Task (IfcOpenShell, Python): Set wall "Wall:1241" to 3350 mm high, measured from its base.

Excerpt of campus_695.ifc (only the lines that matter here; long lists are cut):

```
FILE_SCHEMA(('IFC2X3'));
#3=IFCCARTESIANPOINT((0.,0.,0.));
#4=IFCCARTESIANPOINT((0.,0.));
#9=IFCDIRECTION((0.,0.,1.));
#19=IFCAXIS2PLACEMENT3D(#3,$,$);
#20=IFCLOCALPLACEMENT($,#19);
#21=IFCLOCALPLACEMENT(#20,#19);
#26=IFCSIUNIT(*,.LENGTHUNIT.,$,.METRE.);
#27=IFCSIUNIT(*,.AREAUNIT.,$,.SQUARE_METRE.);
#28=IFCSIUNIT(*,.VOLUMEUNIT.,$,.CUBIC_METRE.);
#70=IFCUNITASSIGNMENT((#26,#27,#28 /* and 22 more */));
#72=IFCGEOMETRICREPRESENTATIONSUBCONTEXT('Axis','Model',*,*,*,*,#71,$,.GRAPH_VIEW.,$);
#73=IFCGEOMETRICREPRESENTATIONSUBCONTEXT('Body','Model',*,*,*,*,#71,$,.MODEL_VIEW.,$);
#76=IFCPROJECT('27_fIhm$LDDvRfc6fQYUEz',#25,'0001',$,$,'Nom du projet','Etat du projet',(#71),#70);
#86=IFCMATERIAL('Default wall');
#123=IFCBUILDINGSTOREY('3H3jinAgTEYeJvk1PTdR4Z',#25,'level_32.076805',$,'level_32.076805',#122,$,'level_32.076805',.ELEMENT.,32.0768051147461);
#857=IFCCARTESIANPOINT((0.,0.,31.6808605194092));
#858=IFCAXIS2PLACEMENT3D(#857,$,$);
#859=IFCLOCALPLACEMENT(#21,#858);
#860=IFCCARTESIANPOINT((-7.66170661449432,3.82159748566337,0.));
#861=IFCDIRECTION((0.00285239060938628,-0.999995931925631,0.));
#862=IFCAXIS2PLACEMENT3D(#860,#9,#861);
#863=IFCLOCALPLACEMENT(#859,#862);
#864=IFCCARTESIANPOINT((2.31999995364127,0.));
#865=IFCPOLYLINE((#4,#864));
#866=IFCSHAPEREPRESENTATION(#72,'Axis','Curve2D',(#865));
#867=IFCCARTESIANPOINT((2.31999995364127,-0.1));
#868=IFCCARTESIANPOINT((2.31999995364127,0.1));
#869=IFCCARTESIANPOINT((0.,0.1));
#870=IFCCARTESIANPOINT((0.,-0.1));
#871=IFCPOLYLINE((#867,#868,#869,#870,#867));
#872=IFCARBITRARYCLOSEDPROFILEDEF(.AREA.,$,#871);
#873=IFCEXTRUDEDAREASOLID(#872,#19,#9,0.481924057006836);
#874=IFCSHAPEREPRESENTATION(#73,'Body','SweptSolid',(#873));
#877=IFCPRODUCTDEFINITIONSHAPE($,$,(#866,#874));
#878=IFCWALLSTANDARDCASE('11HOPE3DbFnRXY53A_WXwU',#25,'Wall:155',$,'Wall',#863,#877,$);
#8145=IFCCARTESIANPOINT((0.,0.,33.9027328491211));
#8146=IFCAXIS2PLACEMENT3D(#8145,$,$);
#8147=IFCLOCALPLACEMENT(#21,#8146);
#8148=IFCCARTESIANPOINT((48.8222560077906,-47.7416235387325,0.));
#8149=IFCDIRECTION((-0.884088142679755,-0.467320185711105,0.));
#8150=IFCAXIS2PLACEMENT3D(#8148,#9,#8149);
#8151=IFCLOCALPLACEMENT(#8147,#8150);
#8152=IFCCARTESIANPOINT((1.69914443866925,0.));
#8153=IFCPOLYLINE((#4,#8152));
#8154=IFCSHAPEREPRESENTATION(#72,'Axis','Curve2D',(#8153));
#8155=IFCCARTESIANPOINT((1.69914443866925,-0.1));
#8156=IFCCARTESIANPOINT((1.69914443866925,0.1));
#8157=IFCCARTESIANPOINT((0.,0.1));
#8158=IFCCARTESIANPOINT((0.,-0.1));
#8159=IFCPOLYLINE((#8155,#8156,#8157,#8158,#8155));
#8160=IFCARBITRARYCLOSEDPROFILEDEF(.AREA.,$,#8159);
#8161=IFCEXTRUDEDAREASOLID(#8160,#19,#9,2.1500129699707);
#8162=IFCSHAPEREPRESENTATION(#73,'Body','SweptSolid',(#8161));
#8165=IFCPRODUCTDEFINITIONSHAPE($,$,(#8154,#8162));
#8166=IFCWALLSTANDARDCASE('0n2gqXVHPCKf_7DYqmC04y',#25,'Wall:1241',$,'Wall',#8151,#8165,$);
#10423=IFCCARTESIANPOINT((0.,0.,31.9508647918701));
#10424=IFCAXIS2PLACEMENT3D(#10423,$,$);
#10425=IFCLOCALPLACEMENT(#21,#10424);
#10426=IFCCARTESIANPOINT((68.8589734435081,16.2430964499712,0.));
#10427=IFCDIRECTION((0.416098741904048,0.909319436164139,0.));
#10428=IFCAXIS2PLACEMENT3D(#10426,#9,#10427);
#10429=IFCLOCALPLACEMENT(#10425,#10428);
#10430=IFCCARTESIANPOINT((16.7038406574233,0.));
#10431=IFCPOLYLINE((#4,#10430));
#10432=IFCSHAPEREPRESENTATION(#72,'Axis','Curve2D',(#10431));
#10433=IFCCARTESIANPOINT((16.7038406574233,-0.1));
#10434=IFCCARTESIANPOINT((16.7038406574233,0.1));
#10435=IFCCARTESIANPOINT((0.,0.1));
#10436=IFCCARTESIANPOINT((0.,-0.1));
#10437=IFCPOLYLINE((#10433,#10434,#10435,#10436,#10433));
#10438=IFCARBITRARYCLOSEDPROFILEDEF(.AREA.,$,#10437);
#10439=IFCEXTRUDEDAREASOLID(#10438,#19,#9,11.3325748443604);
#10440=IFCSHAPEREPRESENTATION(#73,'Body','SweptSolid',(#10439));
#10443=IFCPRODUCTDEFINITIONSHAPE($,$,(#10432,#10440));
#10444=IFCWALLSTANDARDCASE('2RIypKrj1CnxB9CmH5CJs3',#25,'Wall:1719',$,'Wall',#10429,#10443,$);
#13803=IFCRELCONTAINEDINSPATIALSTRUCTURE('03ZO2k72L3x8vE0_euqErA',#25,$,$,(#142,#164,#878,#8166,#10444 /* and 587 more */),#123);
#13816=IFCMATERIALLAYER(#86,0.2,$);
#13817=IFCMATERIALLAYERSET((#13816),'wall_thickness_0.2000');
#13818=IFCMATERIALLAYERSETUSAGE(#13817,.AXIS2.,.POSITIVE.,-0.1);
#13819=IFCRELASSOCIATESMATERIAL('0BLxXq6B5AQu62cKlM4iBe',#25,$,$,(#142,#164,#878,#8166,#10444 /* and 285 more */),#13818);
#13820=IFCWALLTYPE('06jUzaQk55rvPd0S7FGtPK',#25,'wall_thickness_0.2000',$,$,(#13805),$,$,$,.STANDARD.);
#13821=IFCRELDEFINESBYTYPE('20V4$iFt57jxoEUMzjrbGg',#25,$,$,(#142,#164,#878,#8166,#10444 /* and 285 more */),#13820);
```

```python
import ifcopenshell
import ifcopenshell.geom
import ifcopenshell.util.representation
import ifcopenshell.util.shape
import ifcopenshell.util.unit

model = ifcopenshell.open("campus_695.ifc")
unit_scale = ifcopenshell.util.unit.calculate_unit_scale(model)
settings = ifcopenshell.geom.settings()


def volume(element):
    """Net volume in cubic metres, openings subtracted."""
    shape = ifcopenshell.geom.create_shape(settings, element)
    return ifcopenshell.util.shape.get_volume(shape.geometry)


wall = model.by_guid("0n2gqXVHPCKf_7DYqmC04y")
before = volume(wall)

body = ifcopenshell.util.representation.get_representation(wall, "Model", "Body")
solid = body.Items[0]
old_height = solid.Depth
solid.Depth = 3.35 / unit_scale
after = volume(wall)

print(f"height {old_height:g} -> {solid.Depth:g}, volume {before:.3f} -> {after:.3f} m3")

model.write("campus_695_edited.ifc")
```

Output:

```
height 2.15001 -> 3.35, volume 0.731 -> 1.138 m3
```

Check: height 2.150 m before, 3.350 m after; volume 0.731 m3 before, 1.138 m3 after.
